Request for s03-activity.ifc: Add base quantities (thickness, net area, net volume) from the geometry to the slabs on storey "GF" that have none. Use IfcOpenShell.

First a look at what the model holds.

```python
import ifcopenshell
import ifcopenshell.util.element
import ifcopenshell.util.unit

model = ifcopenshell.open("s03-activity.ifc")
print(model.schema)
for unit_type in ("LENGTHUNIT", "AREAUNIT", "VOLUMEUNIT"):
    print(unit_type, ifcopenshell.util.unit.calculate_unit_scale(model, unit_type))
storey = next(s for s in model.by_type("IfcBuildingStorey") if s.Name == "GF")
slabs = [e for e in ifcopenshell.util.element.get_decomposition(storey) if e.is_a("IfcSlab")]
for e in sorted(slabs, key=lambda e: e.id()):
    print(e.id(), e.is_a(), e.Name, list(ifcopenshell.util.element.get_psets(e, qtos_only=True)), sep=" | ")
```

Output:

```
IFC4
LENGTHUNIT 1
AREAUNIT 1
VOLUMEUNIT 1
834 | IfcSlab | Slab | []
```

```python
import ifcopenshell
import ifcopenshell.api.pset
import ifcopenshell.geom
import ifcopenshell.util.element
import ifcopenshell.util.shape
import ifcopenshell.util.unit

model = ifcopenshell.open("s03-activity.ifc")
unit_scale = ifcopenshell.util.unit.calculate_unit_scale(model)
area_scale = ifcopenshell.util.unit.calculate_unit_scale(model, "AREAUNIT")
volume_scale = ifcopenshell.util.unit.calculate_unit_scale(model, "VOLUMEUNIT")
settings = ifcopenshell.geom.settings()

storey = next(s for s in model.by_type("IfcBuildingStorey") if s.Name == "GF")
slabs = [e for e in ifcopenshell.util.element.get_decomposition(storey) if e.is_a("IfcSlab")]

for e in sorted(slabs, key=lambda e: e.id()):
    if ifcopenshell.util.element.get_psets(e, qtos_only=True, should_inherit=False):
        continue
    # Geometry comes back in metres, in the element's own axes.
    shape = ifcopenshell.geom.create_shape(settings, e)
    values = {
        "Width": ifcopenshell.util.shape.get_z(shape.geometry) / unit_scale,
        "NetArea": ifcopenshell.util.shape.get_footprint_area(shape.geometry) / area_scale,
        "NetVolume": ifcopenshell.util.shape.get_volume(shape.geometry) / volume_scale,
    }
    qto = ifcopenshell.api.pset.add_qto(model, product=e, name="Qto_SlabBaseQuantities")
    ifcopenshell.api.pset.edit_qto(model, qto=qto, properties=values)
    print(e.id(), {k: round(v, 3) for k, v in values.items()})

model.write("s03-activity-out.ifc")
```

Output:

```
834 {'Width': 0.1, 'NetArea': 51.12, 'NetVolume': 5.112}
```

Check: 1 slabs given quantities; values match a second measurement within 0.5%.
